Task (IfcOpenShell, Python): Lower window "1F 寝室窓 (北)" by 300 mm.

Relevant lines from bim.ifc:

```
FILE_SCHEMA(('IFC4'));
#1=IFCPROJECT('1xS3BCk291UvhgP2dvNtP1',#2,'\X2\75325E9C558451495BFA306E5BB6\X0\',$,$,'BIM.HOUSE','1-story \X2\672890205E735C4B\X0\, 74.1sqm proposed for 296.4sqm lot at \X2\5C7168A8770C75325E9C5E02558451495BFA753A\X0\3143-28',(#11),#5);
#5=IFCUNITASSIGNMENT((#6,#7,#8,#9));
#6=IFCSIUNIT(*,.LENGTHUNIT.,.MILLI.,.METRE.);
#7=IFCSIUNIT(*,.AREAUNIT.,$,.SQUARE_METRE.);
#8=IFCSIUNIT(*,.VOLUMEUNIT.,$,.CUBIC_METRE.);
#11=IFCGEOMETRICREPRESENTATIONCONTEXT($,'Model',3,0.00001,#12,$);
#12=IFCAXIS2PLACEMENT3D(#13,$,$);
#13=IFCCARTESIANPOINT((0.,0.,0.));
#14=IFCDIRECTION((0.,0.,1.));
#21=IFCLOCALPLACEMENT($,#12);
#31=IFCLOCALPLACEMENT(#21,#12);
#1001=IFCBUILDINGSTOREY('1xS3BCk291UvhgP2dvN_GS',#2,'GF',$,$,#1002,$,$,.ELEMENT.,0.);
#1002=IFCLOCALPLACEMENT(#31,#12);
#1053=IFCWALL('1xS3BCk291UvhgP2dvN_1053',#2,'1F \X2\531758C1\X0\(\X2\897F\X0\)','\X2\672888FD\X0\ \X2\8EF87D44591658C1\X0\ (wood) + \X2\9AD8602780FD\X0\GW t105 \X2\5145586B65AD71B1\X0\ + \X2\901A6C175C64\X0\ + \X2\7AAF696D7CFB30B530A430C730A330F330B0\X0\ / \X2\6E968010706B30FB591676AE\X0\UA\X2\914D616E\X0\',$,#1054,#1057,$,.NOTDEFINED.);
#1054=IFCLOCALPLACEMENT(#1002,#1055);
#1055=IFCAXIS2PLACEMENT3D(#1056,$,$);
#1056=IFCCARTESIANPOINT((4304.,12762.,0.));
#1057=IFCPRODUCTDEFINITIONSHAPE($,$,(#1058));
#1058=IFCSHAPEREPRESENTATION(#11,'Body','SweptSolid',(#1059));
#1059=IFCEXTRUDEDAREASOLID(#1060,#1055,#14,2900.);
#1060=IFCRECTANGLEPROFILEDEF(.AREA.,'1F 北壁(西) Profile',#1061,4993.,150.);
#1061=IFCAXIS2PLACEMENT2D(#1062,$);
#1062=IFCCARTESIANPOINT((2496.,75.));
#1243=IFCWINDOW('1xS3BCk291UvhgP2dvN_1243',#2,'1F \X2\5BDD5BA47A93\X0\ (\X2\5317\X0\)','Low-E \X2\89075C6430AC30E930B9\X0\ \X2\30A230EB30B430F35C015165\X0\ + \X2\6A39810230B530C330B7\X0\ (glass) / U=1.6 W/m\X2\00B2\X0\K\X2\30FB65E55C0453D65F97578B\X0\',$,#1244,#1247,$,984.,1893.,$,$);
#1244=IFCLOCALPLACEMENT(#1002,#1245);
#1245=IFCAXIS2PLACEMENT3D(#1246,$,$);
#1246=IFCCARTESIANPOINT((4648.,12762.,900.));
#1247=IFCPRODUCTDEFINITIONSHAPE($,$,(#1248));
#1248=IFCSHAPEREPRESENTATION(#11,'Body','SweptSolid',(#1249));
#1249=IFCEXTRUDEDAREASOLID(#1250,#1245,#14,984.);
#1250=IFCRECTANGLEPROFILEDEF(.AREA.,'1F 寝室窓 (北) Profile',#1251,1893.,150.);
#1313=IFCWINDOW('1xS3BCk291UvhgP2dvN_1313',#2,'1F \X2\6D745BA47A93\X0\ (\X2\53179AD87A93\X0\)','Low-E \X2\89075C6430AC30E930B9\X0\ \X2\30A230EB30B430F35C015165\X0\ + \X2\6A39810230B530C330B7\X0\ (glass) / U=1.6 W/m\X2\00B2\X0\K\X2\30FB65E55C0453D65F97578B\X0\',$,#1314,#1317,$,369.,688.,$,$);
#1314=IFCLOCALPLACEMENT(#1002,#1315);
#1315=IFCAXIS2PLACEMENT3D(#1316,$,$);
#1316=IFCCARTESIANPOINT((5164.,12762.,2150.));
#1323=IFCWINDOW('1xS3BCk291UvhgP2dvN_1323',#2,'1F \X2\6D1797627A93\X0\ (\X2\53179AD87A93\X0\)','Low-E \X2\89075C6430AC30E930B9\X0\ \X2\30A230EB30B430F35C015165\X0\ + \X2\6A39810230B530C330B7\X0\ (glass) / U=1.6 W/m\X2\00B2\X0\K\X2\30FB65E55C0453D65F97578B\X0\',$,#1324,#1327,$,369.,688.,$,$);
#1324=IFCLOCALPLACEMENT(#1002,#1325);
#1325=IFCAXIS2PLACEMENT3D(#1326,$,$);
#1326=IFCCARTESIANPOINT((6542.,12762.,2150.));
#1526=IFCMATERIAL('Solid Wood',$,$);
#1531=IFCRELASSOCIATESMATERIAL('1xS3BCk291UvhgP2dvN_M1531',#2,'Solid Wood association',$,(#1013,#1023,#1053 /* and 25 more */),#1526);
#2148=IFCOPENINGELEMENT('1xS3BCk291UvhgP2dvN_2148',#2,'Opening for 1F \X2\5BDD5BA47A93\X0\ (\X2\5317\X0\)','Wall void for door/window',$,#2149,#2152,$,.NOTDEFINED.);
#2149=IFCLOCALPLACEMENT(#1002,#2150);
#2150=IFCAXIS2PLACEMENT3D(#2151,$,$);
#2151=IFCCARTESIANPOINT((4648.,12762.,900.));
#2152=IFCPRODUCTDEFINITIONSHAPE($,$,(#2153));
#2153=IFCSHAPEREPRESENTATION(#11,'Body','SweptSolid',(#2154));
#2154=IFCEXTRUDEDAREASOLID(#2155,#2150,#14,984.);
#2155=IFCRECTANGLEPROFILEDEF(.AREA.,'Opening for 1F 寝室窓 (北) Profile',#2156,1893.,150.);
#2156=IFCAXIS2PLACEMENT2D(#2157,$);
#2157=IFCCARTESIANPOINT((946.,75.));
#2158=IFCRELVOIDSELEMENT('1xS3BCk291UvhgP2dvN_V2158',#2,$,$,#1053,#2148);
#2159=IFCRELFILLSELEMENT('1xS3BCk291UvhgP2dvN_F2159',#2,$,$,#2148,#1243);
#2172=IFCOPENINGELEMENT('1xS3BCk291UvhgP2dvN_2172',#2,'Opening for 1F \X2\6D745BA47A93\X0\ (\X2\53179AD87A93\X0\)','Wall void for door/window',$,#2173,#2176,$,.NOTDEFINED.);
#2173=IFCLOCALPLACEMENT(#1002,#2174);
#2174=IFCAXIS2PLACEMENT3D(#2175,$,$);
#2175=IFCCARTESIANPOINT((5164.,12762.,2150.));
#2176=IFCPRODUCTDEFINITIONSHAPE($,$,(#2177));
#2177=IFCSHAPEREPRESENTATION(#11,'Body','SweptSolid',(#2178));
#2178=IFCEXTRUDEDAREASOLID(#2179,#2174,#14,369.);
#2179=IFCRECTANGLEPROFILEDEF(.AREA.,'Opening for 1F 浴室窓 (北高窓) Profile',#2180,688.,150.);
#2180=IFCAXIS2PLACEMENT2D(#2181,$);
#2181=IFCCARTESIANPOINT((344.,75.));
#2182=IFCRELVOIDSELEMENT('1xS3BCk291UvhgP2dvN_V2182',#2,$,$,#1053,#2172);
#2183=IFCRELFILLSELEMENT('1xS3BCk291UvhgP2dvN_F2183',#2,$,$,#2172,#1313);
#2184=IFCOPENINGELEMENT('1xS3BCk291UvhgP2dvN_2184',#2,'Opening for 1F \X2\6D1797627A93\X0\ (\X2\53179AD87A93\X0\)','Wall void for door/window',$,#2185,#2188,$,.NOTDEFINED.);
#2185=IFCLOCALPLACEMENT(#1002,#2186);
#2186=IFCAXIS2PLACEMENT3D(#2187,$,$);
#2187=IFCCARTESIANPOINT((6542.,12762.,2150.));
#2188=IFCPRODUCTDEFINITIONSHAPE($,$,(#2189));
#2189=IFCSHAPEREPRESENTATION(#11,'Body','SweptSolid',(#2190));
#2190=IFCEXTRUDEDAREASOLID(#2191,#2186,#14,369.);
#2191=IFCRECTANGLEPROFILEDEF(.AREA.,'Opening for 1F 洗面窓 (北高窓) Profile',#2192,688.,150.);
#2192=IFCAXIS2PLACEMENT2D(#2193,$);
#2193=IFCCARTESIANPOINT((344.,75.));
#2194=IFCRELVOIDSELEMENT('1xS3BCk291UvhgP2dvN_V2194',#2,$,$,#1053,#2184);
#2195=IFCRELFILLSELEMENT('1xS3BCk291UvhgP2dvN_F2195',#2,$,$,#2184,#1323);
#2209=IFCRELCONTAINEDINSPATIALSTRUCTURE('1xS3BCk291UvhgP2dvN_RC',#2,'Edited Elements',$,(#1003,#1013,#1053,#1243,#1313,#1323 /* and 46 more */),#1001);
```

```python
import numpy as np
import ifcopenshell
import ifcopenshell.api.geometry
import ifcopenshell.util.placement
import ifcopenshell.util.unit

model = ifcopenshell.open("bim.ifc")
unit_scale = ifcopenshell.util.unit.calculate_unit_scale(model)

window = model.by_guid("1xS3BCk291UvhgP2dvN_1243")
opening = window.FillsVoids[0].RelatingOpeningElement
dz = -0.3 / unit_scale

shift = np.array([0.0, 0.0, dz])
# The window is not placed relative to its opening, so move both.
for product in (opening, window):
    matrix = ifcopenshell.util.placement.get_local_placement(product.ObjectPlacement)
    matrix[:3, 3] += shift
    ifcopenshell.api.geometry.edit_object_placement(model, product=product, matrix=matrix, is_si=False)

print(f"moved by {dz * unit_scale:+.3f} m")

model.write("bim_rev.ifc")
```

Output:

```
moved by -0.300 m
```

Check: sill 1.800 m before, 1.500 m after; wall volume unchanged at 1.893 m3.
